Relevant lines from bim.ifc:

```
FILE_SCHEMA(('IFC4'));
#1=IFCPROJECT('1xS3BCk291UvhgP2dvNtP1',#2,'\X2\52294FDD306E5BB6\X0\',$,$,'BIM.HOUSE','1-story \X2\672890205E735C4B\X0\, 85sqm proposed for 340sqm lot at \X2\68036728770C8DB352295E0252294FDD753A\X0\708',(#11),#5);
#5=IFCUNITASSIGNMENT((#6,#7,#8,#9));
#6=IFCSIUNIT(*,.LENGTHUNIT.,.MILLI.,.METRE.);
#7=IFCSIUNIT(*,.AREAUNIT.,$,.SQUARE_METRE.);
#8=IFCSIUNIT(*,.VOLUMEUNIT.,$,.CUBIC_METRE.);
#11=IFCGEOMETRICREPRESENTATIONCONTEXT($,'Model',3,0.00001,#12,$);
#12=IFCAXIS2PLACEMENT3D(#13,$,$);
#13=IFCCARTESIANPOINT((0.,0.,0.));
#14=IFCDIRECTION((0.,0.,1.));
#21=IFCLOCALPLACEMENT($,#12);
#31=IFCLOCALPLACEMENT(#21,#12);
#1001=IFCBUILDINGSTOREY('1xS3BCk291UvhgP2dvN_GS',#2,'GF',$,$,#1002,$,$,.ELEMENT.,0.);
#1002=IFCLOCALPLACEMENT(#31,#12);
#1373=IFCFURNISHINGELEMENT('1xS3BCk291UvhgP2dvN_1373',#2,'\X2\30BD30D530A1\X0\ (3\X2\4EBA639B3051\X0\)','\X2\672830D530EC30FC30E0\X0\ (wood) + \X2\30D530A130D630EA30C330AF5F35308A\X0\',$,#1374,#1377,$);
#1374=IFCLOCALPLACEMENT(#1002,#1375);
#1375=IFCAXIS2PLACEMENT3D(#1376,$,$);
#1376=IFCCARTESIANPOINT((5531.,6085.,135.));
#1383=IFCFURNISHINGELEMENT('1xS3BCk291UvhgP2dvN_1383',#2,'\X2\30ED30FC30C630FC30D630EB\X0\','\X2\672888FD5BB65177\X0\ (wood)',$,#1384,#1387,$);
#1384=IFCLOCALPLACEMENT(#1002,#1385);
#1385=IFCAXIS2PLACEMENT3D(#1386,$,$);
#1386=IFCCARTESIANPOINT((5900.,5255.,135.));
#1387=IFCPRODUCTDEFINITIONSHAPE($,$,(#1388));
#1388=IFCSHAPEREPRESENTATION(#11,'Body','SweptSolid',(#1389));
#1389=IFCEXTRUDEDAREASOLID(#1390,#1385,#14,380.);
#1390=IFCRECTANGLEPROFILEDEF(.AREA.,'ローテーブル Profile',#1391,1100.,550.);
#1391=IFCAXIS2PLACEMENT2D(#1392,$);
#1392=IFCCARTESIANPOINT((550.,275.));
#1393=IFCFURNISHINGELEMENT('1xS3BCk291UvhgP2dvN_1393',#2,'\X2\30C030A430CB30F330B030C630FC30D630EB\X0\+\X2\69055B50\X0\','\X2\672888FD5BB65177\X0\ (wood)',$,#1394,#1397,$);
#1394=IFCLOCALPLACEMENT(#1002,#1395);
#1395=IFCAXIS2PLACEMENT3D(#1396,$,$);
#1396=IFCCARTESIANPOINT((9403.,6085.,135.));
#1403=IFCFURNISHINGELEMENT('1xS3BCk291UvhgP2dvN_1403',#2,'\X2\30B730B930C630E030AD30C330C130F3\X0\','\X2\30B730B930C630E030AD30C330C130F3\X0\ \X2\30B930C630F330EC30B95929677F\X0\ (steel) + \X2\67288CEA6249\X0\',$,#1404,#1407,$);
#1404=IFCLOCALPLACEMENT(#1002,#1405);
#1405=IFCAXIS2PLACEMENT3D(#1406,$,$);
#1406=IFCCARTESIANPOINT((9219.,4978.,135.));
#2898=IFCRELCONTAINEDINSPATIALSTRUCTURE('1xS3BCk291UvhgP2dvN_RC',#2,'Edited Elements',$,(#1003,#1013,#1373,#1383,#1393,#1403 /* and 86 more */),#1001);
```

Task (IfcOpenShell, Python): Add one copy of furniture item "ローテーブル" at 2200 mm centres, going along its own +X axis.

```python
import ifcopenshell
import ifcopenshell.api.geometry
import ifcopenshell.api.root
import ifcopenshell.util.element
import ifcopenshell.util.placement

model = ifcopenshell.open("bim.ifc")


def reuse_history(source, copy):
    """copy_class also copies each property set's owner history, people and application; keep the originals."""
    for rel in copy.IsDefinedBy:
        if rel.is_a("IfcRelDefinesByProperties") and (history := rel.RelatingPropertyDefinition.OwnerHistory):
            rel.RelatingPropertyDefinition.OwnerHistory = source.OwnerHistory
            ifcopenshell.util.element.remove_deep2(model, history)


source = model.by_guid("1xS3BCk291UvhgP2dvN_1383")
base = ifcopenshell.util.placement.get_local_placement(source.ObjectPlacement)
step = base[:3, 0] * 2200.0

for i in range(1, 2):
    copy = ifcopenshell.api.root.copy_class(model, product=source)
    copy.Representation = ifcopenshell.util.element.copy_deep(
        model, source.Representation, exclude=["IfcGeometricRepresentationContext", "IfcRepresentationMap"]
    )
    reuse_history(source, copy)
    matrix = base.copy()
    matrix[:3, 3] += i * step
    print("added at", matrix[:3, 3].round(3) + 0.0)
    ifcopenshell.api.geometry.edit_object_placement(model, product=copy, matrix=matrix, is_si=False)

model.write("bim_edited.ifc")
```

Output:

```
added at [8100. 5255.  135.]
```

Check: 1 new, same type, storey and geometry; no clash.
